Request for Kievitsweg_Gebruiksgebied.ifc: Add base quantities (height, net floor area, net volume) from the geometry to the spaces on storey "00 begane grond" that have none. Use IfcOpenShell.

First a look at what the model holds.

```python
import ifcopenshell
import ifcopenshell.util.element
import ifcopenshell.util.unit

model = ifcopenshell.open("Kievitsweg_Gebruiksgebied.ifc")
print(model.schema)
for unit_type in ("LENGTHUNIT", "AREAUNIT", "VOLUMEUNIT"):
    print(unit_type, ifcopenshell.util.unit.calculate_unit_scale(model, unit_type))
storey = next(s for s in model.by_type("IfcBuildingStorey") if s.Name == "00 begane grond")
spaces = [e for e in ifcopenshell.util.element.get_decomposition(storey) if e.is_a("IfcSpace")]
for e in sorted(spaces, key=lambda e: e.id()):
    print(e.id(), e.is_a(), e.Name, list(ifcopenshell.util.element.get_psets(e, qtos_only=True)), sep=" | ")
```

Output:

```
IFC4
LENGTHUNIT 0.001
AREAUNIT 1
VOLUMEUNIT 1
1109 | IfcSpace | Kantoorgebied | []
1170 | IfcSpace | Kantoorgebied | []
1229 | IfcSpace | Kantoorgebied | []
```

```python
import ifcopenshell
import ifcopenshell.api.pset
import ifcopenshell.geom
import ifcopenshell.util.element
import ifcopenshell.util.shape
import ifcopenshell.util.unit

model = ifcopenshell.open("Kievitsweg_Gebruiksgebied.ifc")
unit_scale = ifcopenshell.util.unit.calculate_unit_scale(model)
area_scale = ifcopenshell.util.unit.calculate_unit_scale(model, "AREAUNIT")
volume_scale = ifcopenshell.util.unit.calculate_unit_scale(model, "VOLUMEUNIT")
settings = ifcopenshell.geom.settings()

storey = next(s for s in model.by_type("IfcBuildingStorey") if s.Name == "00 begane grond")
spaces = [e for e in ifcopenshell.util.element.get_decomposition(storey) if e.is_a("IfcSpace")]

for e in sorted(spaces, key=lambda e: e.id()):
    if ifcopenshell.util.element.get_psets(e, qtos_only=True, should_inherit=False):
        continue
    # Geometry comes back in metres, in the element's own axes.
    shape = ifcopenshell.geom.create_shape(settings, e)
    values = {
        "Height": ifcopenshell.util.shape.get_z(shape.geometry) / unit_scale,
        "NetFloorArea": ifcopenshell.util.shape.get_footprint_area(shape.geometry) / area_scale,
        "NetVolume": ifcopenshell.util.shape.get_volume(shape.geometry) / volume_scale,
    }
    qto = ifcopenshell.api.pset.add_qto(model, product=e, name="Qto_SpaceBaseQuantities")
    ifcopenshell.api.pset.edit_qto(model, qto=qto, properties=values)
    print(e.id(), {k: round(v, 3) for k, v in values.items()})

model.write("Kievitsweg_Gebruiksgebied_rev.ifc")
```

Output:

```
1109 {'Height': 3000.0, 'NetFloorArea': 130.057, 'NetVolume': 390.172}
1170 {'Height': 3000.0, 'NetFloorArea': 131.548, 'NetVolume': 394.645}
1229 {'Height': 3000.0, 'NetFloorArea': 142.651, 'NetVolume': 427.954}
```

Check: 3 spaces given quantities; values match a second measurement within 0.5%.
